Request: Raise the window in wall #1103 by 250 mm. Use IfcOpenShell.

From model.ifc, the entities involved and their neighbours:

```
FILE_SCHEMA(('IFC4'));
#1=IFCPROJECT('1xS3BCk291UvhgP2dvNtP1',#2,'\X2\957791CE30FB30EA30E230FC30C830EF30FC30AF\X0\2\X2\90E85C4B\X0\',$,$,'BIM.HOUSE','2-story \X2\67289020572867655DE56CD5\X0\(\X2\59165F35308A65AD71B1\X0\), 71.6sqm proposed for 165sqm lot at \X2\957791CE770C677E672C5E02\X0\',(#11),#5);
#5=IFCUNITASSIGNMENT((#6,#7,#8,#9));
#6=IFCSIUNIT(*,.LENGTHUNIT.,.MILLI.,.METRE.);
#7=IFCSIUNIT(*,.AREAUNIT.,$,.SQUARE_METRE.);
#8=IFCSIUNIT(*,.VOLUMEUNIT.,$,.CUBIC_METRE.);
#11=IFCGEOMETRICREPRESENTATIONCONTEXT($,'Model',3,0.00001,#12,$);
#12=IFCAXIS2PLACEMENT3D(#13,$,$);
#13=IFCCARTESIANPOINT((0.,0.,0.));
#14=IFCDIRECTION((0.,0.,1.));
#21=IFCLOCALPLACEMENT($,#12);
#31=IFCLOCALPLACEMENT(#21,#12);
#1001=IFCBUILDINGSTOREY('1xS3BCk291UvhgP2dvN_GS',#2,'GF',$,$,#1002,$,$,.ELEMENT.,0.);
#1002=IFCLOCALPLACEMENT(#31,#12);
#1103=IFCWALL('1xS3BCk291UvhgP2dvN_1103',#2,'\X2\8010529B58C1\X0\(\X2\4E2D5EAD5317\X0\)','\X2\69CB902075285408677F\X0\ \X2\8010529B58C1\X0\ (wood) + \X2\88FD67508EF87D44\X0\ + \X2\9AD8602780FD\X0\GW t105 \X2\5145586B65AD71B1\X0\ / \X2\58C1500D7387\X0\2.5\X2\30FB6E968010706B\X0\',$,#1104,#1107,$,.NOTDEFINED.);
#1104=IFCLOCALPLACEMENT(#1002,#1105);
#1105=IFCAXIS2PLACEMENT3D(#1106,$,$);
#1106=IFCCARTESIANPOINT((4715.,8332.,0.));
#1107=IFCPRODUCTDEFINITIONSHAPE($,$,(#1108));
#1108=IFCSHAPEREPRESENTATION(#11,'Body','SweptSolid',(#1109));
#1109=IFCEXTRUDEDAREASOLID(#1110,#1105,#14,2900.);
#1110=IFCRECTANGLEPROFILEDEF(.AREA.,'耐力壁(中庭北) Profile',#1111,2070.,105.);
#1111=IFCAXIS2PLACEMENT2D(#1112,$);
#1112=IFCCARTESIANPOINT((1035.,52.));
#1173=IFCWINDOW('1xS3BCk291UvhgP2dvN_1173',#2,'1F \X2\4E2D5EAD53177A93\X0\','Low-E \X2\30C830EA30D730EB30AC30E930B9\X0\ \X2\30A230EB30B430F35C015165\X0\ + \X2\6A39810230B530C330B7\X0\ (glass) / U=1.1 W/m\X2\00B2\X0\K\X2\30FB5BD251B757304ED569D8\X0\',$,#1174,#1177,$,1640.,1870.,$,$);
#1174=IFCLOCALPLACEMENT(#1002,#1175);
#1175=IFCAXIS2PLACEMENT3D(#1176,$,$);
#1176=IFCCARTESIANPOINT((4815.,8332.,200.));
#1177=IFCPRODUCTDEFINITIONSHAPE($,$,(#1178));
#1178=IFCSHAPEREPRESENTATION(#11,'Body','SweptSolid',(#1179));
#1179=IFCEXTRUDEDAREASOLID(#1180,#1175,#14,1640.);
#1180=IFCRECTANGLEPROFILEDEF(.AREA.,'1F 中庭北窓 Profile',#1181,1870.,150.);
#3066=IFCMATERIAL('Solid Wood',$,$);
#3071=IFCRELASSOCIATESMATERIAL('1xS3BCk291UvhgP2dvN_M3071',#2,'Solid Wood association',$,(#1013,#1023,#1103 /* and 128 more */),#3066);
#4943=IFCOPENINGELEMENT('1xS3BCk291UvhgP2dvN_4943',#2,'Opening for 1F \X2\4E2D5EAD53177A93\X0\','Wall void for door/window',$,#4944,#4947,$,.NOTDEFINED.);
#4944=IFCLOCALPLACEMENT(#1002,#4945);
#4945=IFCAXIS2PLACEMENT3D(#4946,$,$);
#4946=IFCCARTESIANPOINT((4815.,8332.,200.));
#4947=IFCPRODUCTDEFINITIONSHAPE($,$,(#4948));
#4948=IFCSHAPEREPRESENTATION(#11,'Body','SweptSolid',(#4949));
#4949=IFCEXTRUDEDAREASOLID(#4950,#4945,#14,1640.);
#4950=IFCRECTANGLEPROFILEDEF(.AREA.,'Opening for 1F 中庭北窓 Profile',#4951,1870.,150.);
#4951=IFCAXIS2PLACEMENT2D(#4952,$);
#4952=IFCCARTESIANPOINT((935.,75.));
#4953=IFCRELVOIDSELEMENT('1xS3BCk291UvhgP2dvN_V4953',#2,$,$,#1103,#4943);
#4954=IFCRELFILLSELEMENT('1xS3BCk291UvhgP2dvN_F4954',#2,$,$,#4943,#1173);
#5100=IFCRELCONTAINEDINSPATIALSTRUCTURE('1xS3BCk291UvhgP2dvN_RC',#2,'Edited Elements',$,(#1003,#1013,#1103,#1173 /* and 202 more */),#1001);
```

```python
import numpy as np
import ifcopenshell
import ifcopenshell.api.geometry
import ifcopenshell.util.placement
import ifcopenshell.util.unit

model = ifcopenshell.open("model.ifc")
unit_scale = ifcopenshell.util.unit.calculate_unit_scale(model)

window = model.by_guid("1xS3BCk291UvhgP2dvN_1173")
opening = window.FillsVoids[0].RelatingOpeningElement
dz = 250.0

shift = np.array([0.0, 0.0, dz])
# The window is not placed relative to its opening, so move both.
for product in (opening, window):
    matrix = ifcopenshell.util.placement.get_local_placement(product.ObjectPlacement)
    matrix[:3, 3] += shift
    ifcopenshell.api.geometry.edit_object_placement(model, product=product, matrix=matrix, is_si=False)

print(f"moved by {dz * unit_scale:+.3f} m")

model.write("model-out.ifc")
```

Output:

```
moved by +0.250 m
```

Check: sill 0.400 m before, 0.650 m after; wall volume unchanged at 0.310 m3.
